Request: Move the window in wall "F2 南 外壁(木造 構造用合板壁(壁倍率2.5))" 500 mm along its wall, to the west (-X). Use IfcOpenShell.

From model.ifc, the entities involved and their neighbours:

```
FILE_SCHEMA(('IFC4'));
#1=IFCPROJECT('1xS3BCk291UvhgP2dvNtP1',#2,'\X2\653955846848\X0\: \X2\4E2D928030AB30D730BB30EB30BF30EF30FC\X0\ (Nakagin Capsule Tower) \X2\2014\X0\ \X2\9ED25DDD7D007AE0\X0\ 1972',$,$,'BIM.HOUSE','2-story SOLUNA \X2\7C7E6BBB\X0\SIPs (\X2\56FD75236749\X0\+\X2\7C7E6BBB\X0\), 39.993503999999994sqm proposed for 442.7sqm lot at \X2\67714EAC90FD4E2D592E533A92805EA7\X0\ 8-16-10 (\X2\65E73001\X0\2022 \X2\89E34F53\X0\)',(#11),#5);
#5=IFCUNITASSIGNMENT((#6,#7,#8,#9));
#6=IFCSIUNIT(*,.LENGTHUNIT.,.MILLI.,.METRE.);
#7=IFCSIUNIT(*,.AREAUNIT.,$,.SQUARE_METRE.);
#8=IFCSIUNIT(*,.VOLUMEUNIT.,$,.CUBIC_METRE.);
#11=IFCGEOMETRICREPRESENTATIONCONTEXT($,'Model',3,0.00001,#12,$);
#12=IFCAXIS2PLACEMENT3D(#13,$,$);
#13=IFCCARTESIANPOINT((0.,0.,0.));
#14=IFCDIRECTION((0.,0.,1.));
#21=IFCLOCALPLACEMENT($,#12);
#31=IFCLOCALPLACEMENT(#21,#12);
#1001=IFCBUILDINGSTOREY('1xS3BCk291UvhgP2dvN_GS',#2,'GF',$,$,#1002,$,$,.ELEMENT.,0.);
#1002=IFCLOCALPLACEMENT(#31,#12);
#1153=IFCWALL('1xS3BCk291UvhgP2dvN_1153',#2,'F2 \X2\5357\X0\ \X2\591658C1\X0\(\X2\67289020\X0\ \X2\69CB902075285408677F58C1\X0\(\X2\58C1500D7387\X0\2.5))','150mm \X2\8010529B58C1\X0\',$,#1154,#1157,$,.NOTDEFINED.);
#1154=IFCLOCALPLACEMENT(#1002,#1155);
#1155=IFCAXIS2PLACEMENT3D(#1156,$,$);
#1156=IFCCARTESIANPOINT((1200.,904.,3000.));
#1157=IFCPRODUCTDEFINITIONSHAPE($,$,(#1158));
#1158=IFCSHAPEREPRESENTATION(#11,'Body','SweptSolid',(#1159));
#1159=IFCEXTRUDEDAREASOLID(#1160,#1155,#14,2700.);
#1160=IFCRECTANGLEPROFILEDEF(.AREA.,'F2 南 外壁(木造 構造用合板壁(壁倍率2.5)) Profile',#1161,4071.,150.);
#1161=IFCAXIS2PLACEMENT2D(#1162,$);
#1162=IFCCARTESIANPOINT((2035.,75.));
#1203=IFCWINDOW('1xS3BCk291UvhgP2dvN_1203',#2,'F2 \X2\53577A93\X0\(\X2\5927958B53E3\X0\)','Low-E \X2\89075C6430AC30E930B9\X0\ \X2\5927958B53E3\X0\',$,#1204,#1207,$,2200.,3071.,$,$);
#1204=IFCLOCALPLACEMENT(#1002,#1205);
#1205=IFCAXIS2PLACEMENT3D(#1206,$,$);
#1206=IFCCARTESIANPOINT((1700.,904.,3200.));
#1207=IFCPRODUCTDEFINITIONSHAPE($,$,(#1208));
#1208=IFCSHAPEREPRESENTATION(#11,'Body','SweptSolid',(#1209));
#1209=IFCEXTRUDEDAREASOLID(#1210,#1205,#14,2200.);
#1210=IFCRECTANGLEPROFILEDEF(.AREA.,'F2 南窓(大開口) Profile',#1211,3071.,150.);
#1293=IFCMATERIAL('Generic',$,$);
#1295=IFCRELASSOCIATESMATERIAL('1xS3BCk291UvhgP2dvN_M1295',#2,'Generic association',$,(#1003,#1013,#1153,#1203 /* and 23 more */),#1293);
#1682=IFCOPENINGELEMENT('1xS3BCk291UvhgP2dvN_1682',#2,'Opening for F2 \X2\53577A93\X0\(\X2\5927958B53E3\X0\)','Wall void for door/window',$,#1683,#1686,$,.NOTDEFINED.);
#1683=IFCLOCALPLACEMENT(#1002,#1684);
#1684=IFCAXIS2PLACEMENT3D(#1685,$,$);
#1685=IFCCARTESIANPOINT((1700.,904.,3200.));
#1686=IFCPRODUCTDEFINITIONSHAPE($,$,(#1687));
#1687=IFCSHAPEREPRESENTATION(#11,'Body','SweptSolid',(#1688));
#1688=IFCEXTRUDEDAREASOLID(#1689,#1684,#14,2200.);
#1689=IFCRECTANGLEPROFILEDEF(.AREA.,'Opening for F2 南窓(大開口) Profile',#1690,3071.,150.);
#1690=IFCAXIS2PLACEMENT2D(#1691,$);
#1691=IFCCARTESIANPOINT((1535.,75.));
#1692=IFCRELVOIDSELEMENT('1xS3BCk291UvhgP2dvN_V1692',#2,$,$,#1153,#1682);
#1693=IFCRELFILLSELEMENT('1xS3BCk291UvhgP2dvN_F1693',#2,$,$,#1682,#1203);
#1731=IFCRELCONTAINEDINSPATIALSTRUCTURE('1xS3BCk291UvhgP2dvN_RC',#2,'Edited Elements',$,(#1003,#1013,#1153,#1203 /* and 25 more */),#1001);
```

```python
import ifcopenshell
import ifcopenshell.api.geometry
import ifcopenshell.util.placement

model = ifcopenshell.open("model.ifc")

window = model.by_id(1203)
opening = window.FillsVoids[0].RelatingOpeningElement
wall = opening.VoidsElements[0].RelatingBuildingElement

wall_matrix = ifcopenshell.util.placement.get_local_placement(wall.ObjectPlacement)
shift = wall_matrix[:3, 0] * -500.0
before = ifcopenshell.util.placement.get_local_placement(window.ObjectPlacement)[:3, 3].copy()

# The window is not placed relative to its opening, so move both.
for product in (opening, window):
    matrix = ifcopenshell.util.placement.get_local_placement(product.ObjectPlacement)
    matrix[:3, 3] += shift
    ifcopenshell.api.geometry.edit_object_placement(model, product=product, matrix=matrix, is_si=False)

after = ifcopenshell.util.placement.get_local_placement(window.ObjectPlacement)[:3, 3]
print("window moved by", (after - before).round(3) + 0.0)

model.write("model-out.ifc")
```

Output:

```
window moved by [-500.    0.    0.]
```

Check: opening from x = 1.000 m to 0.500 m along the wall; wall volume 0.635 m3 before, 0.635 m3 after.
